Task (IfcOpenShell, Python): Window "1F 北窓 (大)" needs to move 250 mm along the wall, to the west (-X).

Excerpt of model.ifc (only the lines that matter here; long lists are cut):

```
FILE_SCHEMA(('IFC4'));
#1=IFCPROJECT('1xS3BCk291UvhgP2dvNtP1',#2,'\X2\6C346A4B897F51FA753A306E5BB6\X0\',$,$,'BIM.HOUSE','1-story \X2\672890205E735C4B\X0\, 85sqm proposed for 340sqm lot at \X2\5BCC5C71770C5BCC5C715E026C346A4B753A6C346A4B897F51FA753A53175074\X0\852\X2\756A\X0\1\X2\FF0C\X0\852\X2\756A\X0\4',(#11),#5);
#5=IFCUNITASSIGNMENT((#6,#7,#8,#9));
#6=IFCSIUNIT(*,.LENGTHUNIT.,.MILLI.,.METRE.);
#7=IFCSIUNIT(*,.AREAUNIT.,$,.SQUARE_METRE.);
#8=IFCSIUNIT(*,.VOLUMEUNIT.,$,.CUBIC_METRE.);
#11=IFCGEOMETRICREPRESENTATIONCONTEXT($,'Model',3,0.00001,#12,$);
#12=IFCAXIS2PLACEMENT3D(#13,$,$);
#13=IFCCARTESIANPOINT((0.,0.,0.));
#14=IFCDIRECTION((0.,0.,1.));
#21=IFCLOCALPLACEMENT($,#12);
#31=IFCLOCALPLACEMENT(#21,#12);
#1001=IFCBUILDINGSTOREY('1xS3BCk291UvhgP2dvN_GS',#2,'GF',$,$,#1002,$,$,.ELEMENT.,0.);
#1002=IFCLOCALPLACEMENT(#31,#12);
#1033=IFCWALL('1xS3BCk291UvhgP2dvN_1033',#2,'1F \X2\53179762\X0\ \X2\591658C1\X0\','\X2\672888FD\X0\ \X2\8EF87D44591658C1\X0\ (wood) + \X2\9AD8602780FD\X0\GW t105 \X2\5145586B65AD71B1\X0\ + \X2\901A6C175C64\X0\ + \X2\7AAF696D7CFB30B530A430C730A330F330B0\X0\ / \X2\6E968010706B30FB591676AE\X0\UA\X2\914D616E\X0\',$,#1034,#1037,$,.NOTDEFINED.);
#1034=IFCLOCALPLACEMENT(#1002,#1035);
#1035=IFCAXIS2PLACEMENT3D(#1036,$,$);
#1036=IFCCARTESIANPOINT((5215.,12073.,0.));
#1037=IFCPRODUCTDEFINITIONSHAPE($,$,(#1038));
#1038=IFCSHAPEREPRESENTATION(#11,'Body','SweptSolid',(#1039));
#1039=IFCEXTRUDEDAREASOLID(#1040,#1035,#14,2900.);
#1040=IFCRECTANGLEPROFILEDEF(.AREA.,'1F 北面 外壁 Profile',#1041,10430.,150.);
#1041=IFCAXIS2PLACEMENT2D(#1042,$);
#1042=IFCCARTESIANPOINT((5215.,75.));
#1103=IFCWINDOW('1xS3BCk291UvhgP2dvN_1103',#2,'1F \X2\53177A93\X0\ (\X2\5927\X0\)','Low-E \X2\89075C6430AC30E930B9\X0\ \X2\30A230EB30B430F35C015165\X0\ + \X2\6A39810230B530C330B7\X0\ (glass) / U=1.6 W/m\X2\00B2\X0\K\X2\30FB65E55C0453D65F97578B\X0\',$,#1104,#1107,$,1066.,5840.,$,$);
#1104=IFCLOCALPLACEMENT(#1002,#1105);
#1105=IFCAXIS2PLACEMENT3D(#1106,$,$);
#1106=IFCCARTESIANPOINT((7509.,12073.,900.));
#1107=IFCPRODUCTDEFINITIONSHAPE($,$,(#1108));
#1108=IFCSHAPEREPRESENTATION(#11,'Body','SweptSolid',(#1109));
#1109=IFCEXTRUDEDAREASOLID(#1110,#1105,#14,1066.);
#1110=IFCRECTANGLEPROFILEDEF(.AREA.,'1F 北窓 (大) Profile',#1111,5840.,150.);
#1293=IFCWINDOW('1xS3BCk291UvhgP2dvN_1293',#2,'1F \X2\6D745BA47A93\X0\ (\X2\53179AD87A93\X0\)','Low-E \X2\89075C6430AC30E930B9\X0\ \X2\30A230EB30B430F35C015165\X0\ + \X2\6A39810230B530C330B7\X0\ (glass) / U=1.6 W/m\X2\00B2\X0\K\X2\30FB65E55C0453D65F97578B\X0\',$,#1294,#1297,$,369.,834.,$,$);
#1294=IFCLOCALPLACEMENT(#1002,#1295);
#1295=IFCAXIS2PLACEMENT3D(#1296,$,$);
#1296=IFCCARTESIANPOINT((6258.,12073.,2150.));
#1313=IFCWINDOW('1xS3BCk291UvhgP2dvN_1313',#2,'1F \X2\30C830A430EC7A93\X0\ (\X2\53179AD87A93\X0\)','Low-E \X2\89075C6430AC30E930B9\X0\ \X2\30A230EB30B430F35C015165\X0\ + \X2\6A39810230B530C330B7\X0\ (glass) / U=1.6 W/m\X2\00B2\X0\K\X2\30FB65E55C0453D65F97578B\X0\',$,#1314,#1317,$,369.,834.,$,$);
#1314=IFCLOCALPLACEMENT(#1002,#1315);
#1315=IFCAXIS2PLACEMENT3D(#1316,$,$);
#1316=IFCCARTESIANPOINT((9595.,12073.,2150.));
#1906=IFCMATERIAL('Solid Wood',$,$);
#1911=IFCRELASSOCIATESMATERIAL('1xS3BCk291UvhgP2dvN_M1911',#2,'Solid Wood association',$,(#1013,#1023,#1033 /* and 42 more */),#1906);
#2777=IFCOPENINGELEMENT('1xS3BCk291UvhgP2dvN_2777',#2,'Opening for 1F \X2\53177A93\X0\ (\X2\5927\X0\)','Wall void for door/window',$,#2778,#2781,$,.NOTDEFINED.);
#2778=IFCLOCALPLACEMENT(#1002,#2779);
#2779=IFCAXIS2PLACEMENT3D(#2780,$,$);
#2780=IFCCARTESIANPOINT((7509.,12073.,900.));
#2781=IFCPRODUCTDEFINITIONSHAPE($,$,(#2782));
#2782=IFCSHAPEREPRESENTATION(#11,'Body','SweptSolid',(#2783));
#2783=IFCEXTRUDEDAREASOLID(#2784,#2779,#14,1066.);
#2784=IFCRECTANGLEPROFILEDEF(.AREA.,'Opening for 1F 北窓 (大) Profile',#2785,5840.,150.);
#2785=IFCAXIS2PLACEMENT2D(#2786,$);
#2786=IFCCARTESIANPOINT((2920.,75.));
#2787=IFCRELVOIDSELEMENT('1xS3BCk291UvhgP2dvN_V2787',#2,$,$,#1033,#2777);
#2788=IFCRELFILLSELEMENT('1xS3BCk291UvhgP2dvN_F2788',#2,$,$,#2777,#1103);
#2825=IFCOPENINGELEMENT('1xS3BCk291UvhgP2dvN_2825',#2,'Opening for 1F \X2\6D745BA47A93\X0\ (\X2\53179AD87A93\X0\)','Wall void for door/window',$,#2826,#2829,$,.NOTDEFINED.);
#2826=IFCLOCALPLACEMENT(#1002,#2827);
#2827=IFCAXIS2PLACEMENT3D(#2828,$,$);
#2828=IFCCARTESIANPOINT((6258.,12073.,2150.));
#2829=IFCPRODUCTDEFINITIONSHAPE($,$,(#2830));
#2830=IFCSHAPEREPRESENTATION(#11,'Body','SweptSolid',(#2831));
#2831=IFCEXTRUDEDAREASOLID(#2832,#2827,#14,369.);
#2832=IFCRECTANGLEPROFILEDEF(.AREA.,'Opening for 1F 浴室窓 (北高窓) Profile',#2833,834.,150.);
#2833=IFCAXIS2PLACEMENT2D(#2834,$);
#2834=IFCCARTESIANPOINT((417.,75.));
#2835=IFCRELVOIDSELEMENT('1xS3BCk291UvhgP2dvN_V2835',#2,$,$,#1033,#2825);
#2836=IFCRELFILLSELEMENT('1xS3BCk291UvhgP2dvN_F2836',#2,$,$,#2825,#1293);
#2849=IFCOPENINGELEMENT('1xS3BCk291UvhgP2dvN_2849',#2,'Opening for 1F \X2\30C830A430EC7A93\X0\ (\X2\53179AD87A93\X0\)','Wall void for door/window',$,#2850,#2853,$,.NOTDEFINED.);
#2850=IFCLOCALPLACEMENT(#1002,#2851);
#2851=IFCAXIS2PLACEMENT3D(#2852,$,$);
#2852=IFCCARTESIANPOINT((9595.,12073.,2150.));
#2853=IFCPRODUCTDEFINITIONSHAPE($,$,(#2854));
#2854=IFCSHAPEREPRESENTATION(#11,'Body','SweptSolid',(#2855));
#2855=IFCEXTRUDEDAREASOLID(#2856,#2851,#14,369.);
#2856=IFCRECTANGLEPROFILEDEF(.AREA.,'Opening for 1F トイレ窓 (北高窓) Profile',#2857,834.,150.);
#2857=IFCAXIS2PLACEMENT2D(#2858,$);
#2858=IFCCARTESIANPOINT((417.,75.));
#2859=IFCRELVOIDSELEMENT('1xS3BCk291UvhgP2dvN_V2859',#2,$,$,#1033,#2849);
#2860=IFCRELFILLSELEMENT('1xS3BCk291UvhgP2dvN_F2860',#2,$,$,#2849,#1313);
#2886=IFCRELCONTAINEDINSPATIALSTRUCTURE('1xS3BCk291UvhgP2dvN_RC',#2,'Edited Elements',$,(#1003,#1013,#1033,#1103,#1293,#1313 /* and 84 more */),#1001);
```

```python
import ifcopenshell
import ifcopenshell.api.geometry
import ifcopenshell.util.placement

model = ifcopenshell.open("model.ifc")

window = model.by_guid("1xS3BCk291UvhgP2dvN_1103")
opening = window.FillsVoids[0].RelatingOpeningElement
wall = opening.VoidsElements[0].RelatingBuildingElement

wall_matrix = ifcopenshell.util.placement.get_local_placement(wall.ObjectPlacement)
shift = wall_matrix[:3, 0] * -250.0
before = ifcopenshell.util.placement.get_local_placement(window.ObjectPlacement)[:3, 3].copy()

# The window is not placed relative to its opening, so move both.
for product in (opening, window):
    matrix = ifcopenshell.util.placement.get_local_placement(product.ObjectPlacement)
    matrix[:3, 3] += shift
    ifcopenshell.api.geometry.edit_object_placement(model, product=product, matrix=matrix, is_si=False)

after = ifcopenshell.util.placement.get_local_placement(window.ObjectPlacement)[:3, 3]
print("window moved by", (after - before).round(3) + 0.0)

model.write("model_v2.ifc")
```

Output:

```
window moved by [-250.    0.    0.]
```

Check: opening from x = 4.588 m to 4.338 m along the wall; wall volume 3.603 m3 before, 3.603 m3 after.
